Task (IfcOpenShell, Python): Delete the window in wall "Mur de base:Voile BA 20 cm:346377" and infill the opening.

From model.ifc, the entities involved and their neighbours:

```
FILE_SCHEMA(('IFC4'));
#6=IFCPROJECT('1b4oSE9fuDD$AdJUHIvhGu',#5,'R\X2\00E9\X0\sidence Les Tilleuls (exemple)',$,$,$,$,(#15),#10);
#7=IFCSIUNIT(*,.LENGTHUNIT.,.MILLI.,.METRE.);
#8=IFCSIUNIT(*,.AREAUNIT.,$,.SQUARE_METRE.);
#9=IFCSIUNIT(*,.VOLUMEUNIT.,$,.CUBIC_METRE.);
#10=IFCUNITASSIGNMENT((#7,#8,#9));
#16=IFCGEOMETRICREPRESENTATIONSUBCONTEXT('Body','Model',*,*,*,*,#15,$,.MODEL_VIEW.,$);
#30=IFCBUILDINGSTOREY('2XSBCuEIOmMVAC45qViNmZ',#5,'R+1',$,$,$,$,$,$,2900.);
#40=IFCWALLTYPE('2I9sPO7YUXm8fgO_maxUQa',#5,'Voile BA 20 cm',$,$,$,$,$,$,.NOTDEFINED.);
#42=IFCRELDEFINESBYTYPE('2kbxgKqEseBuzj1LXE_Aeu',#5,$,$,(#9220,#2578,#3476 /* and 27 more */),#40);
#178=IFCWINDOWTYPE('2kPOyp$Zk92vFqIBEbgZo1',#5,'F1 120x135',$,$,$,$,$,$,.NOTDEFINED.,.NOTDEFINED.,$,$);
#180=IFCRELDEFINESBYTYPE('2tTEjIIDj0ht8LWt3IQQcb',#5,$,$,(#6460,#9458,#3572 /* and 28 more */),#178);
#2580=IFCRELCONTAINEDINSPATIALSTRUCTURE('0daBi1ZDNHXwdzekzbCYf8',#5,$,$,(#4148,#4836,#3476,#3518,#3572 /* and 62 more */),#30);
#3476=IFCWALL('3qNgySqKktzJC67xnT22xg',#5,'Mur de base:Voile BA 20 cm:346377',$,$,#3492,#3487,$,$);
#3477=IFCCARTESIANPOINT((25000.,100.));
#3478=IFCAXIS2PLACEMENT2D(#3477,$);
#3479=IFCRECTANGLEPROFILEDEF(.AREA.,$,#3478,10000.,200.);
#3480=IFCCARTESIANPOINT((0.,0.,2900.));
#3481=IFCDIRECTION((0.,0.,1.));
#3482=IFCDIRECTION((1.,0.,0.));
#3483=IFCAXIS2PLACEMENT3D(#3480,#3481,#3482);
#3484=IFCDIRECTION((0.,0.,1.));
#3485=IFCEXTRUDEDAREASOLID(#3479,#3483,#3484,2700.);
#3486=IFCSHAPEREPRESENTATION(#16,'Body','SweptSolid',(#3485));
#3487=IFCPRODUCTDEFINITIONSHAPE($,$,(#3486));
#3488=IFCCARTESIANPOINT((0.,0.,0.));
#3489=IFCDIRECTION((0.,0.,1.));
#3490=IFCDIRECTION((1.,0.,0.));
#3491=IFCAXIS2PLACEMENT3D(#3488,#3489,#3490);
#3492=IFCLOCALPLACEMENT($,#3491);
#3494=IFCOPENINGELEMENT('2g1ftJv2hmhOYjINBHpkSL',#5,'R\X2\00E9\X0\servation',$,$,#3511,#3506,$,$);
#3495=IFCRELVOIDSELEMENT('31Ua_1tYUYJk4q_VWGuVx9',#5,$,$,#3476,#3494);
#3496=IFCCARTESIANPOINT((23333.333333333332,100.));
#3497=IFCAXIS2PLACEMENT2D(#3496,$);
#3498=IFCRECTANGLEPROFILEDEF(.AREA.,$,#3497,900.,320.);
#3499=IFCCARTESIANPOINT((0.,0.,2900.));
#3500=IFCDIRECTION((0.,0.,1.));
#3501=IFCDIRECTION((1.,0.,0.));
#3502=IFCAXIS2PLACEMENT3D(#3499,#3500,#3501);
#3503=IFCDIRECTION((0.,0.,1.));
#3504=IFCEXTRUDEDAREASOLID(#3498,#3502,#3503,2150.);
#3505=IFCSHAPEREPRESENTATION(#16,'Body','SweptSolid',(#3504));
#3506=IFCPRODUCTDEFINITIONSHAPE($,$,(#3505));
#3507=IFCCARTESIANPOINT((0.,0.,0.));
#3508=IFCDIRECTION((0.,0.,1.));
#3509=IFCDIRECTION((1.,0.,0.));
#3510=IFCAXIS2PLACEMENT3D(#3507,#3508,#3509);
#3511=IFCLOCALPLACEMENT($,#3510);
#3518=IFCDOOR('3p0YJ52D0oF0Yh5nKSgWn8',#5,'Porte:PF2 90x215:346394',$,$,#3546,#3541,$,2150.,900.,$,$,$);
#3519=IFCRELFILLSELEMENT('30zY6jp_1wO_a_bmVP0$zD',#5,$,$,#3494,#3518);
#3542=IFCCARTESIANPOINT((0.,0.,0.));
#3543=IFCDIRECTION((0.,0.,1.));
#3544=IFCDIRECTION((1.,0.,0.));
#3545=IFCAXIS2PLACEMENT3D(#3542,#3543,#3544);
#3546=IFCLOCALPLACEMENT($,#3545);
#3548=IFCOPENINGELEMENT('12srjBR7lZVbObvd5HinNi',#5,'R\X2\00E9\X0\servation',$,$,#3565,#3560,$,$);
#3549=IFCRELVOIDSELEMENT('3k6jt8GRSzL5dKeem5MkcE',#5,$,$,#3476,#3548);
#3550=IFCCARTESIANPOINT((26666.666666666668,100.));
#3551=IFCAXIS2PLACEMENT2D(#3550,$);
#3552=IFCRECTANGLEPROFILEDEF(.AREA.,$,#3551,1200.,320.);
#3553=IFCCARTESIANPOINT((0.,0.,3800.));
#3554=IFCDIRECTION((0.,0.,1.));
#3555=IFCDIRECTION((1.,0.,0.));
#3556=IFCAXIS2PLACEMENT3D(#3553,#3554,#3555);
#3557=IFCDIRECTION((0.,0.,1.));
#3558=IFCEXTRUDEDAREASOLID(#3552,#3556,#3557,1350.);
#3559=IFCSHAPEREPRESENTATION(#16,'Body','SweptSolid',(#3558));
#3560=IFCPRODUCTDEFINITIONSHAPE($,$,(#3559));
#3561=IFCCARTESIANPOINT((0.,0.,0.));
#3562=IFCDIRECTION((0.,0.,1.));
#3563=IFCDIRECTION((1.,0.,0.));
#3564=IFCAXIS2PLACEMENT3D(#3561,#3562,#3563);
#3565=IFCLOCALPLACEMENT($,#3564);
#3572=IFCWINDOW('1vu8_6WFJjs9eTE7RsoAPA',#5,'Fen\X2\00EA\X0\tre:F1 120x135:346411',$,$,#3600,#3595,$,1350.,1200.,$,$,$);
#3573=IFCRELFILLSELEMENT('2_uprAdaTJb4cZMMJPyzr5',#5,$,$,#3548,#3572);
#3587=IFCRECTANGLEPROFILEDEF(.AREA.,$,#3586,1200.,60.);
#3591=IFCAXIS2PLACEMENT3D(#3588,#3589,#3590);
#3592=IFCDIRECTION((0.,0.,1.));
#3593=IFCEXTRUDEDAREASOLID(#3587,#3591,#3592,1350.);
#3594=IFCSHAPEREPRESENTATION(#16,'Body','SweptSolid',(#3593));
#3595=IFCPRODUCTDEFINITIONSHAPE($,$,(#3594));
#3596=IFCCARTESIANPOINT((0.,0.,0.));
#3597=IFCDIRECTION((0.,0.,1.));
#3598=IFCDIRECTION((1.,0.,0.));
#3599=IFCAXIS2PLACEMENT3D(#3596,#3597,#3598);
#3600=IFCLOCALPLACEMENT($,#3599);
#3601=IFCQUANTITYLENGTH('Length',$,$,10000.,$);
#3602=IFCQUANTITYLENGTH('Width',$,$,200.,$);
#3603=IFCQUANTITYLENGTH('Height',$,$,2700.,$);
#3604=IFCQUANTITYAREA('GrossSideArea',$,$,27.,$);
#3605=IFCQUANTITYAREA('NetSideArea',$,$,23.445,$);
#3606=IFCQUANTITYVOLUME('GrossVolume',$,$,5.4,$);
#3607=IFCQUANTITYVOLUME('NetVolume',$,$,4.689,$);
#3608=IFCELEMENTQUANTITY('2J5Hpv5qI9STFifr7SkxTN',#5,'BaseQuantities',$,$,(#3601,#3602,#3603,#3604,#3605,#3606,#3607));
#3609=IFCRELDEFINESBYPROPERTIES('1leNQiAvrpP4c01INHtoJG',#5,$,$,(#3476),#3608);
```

```python
import ifcopenshell
import ifcopenshell.api.feature
import ifcopenshell.api.pset
import ifcopenshell.api.root
import ifcopenshell.geom
import ifcopenshell.util.element
import ifcopenshell.util.shape
import ifcopenshell.util.unit

model = ifcopenshell.open("model.ifc")
area_scale = ifcopenshell.util.unit.calculate_unit_scale(model, "AREAUNIT")
volume_scale = ifcopenshell.util.unit.calculate_unit_scale(model, "VOLUMEUNIT")
settings = ifcopenshell.geom.settings()


def volume(element):
    """Net volume in cubic metres, openings subtracted."""
    shape = ifcopenshell.geom.create_shape(settings, element)
    return ifcopenshell.util.shape.get_volume(shape.geometry)


window = model.by_guid("1vu8_6WFJjs9eTE7RsoAPA")
opening = window.FillsVoids[0].RelatingOpeningElement
wall = opening.VoidsElements[0].RelatingBuildingElement
before = volume(wall)

ifcopenshell.api.root.remove_product(model, product=window)
ifcopenshell.api.feature.remove_feature(model, feature=opening)

after = volume(wall)
thickness = 0.2  # wall thickness in metres

# Update the wall's stored quantities.
qto = model.by_id(ifcopenshell.util.element.get_pset(wall, "BaseQuantities", should_inherit=False)["id"])
ifcopenshell.api.pset.edit_qto(model, qto=qto, properties={
    "NetSideArea": after / thickness / area_scale,
    "NetVolume": after / volume_scale,
})

print(f"wall volume {before:.3f} -> {after:.3f} m3")

model.write("model_v2.ifc")
```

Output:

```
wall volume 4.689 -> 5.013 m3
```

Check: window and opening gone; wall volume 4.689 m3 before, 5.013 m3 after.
